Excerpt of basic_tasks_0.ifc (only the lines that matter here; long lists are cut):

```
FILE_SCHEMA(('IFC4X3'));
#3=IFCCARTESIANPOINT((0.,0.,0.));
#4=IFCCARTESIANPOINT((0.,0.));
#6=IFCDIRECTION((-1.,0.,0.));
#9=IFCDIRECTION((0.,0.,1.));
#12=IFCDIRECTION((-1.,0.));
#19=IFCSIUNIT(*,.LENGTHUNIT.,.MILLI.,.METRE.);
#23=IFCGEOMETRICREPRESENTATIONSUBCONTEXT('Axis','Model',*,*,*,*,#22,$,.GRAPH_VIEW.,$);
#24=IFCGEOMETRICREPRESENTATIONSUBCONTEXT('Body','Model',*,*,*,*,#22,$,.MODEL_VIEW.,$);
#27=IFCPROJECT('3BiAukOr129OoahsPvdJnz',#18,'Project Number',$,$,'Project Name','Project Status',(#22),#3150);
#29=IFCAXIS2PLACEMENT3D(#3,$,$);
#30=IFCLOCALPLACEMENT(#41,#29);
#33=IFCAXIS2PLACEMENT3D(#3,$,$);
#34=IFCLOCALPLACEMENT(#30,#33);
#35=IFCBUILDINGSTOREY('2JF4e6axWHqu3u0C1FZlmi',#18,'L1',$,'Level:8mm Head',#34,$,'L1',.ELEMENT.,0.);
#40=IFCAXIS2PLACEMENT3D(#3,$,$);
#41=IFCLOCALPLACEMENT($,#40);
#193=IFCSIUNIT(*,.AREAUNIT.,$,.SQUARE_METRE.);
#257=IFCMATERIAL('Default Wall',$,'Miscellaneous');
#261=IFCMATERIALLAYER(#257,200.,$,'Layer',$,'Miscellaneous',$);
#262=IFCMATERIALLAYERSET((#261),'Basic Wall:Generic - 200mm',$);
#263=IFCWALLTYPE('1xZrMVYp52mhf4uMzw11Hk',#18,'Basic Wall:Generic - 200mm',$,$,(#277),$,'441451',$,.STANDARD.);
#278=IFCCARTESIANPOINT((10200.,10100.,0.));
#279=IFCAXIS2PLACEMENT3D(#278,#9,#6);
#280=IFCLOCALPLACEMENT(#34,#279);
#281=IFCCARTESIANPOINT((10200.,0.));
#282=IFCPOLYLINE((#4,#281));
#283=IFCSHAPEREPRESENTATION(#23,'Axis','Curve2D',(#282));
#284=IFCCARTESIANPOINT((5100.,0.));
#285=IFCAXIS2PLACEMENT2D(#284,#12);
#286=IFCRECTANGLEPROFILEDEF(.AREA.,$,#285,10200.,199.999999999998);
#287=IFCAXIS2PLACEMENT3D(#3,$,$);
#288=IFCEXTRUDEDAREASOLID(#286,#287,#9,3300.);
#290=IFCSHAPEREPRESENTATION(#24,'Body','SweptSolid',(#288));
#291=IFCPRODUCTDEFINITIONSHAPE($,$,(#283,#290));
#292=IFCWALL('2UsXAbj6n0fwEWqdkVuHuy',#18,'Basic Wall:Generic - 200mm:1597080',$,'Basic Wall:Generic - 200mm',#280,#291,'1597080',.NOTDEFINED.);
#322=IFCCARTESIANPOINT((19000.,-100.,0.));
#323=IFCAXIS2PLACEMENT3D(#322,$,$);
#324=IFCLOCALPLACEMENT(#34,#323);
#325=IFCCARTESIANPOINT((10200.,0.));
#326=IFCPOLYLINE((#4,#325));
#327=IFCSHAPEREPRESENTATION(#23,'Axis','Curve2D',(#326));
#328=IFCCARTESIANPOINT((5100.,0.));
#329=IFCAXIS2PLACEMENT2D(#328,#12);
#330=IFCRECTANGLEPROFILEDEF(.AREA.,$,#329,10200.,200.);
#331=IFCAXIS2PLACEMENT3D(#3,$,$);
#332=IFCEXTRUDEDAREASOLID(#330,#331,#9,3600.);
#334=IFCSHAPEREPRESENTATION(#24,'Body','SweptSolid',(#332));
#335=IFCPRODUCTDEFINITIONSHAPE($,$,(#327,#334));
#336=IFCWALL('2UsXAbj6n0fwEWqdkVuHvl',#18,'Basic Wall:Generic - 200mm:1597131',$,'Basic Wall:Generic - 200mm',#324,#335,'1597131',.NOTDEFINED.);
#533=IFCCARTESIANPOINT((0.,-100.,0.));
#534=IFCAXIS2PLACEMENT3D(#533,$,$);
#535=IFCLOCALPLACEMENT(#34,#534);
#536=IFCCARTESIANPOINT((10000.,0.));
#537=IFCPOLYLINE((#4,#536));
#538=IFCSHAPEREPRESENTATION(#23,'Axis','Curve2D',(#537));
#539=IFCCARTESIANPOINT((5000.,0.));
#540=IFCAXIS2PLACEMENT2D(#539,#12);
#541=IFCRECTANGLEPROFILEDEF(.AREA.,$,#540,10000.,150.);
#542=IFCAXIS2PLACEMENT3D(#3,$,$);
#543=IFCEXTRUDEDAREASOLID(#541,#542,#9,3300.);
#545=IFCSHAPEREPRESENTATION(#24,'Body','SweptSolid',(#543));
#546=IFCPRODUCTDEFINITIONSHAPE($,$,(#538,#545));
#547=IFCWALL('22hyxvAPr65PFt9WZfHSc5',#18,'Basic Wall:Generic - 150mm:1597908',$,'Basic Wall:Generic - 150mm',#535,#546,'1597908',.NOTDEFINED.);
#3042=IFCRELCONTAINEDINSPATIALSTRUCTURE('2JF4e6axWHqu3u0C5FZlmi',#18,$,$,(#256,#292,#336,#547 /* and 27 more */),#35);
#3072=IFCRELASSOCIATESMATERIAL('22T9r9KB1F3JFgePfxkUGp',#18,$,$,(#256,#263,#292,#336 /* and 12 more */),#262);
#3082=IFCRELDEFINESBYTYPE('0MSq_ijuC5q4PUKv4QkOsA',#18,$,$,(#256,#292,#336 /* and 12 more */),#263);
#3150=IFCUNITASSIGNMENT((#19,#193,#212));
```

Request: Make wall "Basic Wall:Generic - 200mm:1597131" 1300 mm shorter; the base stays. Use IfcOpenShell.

```python
import ifcopenshell
import ifcopenshell.geom
import ifcopenshell.util.representation
import ifcopenshell.util.shape
import ifcopenshell.util.unit

model = ifcopenshell.open("basic_tasks_0.ifc")
unit_scale = ifcopenshell.util.unit.calculate_unit_scale(model)
settings = ifcopenshell.geom.settings()


def volume(element):
    """Net volume in cubic metres, openings subtracted."""
    shape = ifcopenshell.geom.create_shape(settings, element)
    return ifcopenshell.util.shape.get_volume(shape.geometry)


wall = model.by_guid("2UsXAbj6n0fwEWqdkVuHvl")
before = volume(wall)

body = ifcopenshell.util.representation.get_representation(wall, "Model", "Body")
solid = body.Items[0]
old_height = solid.Depth
solid.Depth -= 1.3 / unit_scale
after = volume(wall)

print(f"height {old_height:g} -> {solid.Depth:g}, volume {before:.3f} -> {after:.3f} m3")

model.write("basic_tasks_0_edited.ifc")
```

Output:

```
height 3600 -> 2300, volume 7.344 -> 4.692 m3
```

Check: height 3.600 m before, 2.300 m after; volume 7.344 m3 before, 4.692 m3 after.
